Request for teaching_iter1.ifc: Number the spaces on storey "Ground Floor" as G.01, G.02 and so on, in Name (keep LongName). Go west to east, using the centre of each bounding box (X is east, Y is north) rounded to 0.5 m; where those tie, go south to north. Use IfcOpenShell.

First a look at what the model holds.

```python
import ifcopenshell
import ifcopenshell.util.element
import ifcopenshell.util.placement

model = ifcopenshell.open("teaching_iter1.ifc")
print(model.schema)
storey = next(s for s in model.by_type("IfcBuildingStorey") if s.Name == "Ground Floor")
spaces = [e for e in ifcopenshell.util.element.get_decomposition(storey) if e.is_a("IfcSpace")]
for e in sorted(spaces, key=lambda e: e.id()):
    origin = ifcopenshell.util.placement.get_local_placement(e.ObjectPlacement)[:3, 3]
    print(e.id(), e.Name, e.LongName, origin.round(2) + 0.0, sep=" | ")
```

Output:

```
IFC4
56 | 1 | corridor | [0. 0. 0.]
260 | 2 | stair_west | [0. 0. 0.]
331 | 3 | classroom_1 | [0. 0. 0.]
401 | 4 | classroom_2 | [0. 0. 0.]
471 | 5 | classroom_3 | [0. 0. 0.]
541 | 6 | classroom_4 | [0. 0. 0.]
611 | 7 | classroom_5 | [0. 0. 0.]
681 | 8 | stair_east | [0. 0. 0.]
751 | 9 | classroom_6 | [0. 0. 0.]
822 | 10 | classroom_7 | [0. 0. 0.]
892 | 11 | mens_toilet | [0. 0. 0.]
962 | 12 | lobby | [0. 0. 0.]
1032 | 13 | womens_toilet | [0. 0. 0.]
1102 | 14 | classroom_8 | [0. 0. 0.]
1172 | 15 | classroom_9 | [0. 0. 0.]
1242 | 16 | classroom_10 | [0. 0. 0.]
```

```python
import ifcopenshell
import ifcopenshell.geom
import ifcopenshell.util.element
import ifcopenshell.util.shape

model = ifcopenshell.open("teaching_iter1.ifc")
settings = ifcopenshell.geom.settings()
settings.set("use-world-coords", True)


def centre(element):
    shape = ifcopenshell.geom.create_shape(settings, element)
    return ifcopenshell.util.shape.get_bbox_centroid(shape.geometry)


storey = next(s for s in model.by_type("IfcBuildingStorey") if s.Name == "Ground Floor")
spaces = [e for e in ifcopenshell.util.element.get_decomposition(storey) if e.is_a("IfcSpace")]

# Insertion points can sit at a corner or the storey origin, so sort by the geometry (in metres).
centres = {e: centre(e) for e in spaces}
spaces.sort(key=lambda e: (round(centres[e][0] / 0.5), centres[e][1]))

for i, e in enumerate(spaces, start=1):
    number = f"G.{i:02d}"
    e.Name = number
    print(e.id(), number)

model.write("teaching_iter1_edited.ifc")
```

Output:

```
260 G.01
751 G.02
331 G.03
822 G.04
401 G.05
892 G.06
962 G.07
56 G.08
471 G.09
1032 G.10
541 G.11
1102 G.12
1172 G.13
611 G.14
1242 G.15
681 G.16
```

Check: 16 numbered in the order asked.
